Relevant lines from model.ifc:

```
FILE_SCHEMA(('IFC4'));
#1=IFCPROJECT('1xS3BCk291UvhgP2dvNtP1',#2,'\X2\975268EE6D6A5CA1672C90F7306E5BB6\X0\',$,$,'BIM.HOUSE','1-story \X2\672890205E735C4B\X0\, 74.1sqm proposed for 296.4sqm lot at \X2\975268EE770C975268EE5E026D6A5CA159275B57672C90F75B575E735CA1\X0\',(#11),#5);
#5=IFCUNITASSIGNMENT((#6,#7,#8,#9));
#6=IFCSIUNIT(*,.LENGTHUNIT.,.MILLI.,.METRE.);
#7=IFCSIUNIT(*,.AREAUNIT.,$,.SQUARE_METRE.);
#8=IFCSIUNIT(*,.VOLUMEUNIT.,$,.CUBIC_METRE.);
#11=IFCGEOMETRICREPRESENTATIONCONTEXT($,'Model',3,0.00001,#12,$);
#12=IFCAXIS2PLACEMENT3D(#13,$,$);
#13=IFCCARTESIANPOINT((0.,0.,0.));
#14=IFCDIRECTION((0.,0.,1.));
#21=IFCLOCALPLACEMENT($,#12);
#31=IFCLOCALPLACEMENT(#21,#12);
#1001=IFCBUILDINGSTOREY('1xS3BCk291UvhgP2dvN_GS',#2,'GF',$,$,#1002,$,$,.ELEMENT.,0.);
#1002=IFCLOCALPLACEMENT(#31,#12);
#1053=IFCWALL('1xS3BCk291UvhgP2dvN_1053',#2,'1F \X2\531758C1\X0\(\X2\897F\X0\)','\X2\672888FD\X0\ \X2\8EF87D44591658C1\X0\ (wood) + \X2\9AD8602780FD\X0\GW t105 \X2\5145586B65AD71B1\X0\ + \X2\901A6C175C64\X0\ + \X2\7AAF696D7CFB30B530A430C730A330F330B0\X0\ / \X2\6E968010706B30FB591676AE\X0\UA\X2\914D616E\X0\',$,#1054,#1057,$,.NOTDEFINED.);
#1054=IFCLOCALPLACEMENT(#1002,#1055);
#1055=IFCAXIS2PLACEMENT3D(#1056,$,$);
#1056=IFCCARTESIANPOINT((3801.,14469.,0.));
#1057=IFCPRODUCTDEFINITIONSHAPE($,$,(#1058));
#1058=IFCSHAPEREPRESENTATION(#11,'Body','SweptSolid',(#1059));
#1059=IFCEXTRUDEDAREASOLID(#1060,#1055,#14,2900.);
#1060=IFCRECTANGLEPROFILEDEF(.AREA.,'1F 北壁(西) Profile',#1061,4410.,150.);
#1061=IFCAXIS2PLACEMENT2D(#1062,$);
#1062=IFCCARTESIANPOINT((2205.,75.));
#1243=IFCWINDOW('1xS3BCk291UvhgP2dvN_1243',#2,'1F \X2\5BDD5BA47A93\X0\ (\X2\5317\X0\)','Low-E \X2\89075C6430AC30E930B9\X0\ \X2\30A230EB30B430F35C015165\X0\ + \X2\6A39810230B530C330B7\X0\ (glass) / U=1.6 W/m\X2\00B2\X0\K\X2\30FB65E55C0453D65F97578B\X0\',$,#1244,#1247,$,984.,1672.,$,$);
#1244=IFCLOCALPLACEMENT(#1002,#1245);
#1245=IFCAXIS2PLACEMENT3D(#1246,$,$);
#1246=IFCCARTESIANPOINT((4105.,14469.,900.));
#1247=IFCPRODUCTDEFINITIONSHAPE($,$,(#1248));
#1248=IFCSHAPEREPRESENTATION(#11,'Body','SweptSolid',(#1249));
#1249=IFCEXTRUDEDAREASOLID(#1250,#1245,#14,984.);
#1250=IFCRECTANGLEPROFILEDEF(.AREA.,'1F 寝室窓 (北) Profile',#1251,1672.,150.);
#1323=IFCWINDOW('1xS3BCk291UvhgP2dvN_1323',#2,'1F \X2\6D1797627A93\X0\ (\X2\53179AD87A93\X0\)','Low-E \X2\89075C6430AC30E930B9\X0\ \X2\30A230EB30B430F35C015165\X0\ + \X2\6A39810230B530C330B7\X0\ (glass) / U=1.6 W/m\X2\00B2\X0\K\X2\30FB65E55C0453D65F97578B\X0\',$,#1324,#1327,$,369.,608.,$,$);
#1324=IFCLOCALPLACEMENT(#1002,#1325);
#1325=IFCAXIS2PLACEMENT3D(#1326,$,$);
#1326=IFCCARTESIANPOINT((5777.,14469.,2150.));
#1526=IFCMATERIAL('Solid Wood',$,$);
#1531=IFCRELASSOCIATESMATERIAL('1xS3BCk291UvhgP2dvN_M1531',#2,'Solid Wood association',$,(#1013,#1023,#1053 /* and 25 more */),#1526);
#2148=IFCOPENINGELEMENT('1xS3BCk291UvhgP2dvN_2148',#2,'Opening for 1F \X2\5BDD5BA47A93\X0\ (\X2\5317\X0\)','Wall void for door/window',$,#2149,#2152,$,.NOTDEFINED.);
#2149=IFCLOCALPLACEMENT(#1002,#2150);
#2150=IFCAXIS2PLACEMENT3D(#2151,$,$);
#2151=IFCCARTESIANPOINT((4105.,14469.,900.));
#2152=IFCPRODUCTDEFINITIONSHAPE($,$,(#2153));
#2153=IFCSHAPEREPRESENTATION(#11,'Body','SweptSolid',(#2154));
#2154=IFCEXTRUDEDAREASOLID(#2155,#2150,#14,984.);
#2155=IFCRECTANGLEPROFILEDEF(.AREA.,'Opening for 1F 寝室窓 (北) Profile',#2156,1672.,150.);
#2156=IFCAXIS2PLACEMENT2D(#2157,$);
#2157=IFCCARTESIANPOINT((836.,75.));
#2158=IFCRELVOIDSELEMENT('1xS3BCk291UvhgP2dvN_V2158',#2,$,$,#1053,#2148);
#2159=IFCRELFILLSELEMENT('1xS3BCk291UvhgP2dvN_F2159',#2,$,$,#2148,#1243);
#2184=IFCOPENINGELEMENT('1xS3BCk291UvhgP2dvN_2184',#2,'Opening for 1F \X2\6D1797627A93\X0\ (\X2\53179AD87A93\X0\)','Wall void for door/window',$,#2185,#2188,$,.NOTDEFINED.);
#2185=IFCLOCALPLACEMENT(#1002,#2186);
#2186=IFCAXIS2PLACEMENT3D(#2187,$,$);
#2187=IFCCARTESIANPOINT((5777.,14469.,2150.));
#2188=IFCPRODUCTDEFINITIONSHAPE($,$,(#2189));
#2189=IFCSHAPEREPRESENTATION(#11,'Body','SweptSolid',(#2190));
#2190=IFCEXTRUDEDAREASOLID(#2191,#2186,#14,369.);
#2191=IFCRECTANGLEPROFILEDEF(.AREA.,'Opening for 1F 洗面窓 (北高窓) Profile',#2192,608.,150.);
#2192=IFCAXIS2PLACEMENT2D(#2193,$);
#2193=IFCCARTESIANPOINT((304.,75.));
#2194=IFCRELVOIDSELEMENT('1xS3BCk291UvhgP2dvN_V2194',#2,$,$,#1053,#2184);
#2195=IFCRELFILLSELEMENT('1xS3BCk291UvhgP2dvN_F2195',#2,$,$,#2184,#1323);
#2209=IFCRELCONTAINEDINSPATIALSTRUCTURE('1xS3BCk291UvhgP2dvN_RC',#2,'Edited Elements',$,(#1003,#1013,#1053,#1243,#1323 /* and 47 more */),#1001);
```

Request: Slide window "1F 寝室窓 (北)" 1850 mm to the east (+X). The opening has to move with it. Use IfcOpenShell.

```python
import ifcopenshell
import ifcopenshell.api.geometry
import ifcopenshell.util.placement
import ifcopenshell.util.unit

model = ifcopenshell.open("model.ifc")
unit_scale = ifcopenshell.util.unit.calculate_unit_scale(model)

window = model.by_guid("1xS3BCk291UvhgP2dvN_1243")
opening = window.FillsVoids[0].RelatingOpeningElement
wall = opening.VoidsElements[0].RelatingBuildingElement

wall_matrix = ifcopenshell.util.placement.get_local_placement(wall.ObjectPlacement)
shift = wall_matrix[:3, 0] * 1.85 / unit_scale
before = ifcopenshell.util.placement.get_local_placement(window.ObjectPlacement)[:3, 3].copy()

# The window is not placed relative to its opening, so move both.
for product in (opening, window):
    matrix = ifcopenshell.util.placement.get_local_placement(product.ObjectPlacement)
    matrix[:3, 3] += shift
    ifcopenshell.api.geometry.edit_object_placement(model, product=product, matrix=matrix, is_si=False)

after = ifcopenshell.util.placement.get_local_placement(window.ObjectPlacement)[:3, 3]
print("window moved by", (after - before).round(3) + 0.0)

model.write("model_rev.ifc")
```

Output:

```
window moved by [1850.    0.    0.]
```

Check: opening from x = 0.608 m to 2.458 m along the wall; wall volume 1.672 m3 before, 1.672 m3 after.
